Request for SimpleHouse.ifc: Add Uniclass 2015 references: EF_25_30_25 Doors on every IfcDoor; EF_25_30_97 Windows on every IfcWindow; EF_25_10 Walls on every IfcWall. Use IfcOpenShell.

First a look at what the model holds.

```python
import ifcopenshell

model = ifcopenshell.open("SimpleHouse.ifc")
print(model.schema)
print("classifications:", [c.Name for c in model.by_type("IfcClassification")])
for ifc_class in ("IfcDoor", "IfcRoof", "IfcStair", "IfcWall", "IfcWindow"):
    print(ifc_class, len(model.by_type(ifc_class)))
```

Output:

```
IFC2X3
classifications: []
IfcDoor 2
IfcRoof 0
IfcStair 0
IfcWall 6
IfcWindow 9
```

```python
import ifcopenshell
import ifcopenshell.api.classification

model = ifcopenshell.open("SimpleHouse.ifc")

# IFC2X3 requires Source and Edition and has no link from the project to the system.
system = model.create_entity("IfcClassification", Source="NBS", Edition="2015", Name="Uniclass 2015")

codes = {
    "IfcDoor": ("EF_25_30_25", "Doors"),
    "IfcWindow": ("EF_25_30_97", "Windows"),
    "IfcWall": ("EF_25_10", "Walls"),
}
for ifc_class, (code, name) in codes.items():
    products = model.by_type(ifc_class)
    ifcopenshell.api.classification.add_reference(
        model, products=products, classification=system, identification=code, name=name
    )
    print(code, len(products))

model.write("SimpleHouse_edited.ifc")
```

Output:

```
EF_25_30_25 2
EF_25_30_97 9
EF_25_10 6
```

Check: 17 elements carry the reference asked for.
